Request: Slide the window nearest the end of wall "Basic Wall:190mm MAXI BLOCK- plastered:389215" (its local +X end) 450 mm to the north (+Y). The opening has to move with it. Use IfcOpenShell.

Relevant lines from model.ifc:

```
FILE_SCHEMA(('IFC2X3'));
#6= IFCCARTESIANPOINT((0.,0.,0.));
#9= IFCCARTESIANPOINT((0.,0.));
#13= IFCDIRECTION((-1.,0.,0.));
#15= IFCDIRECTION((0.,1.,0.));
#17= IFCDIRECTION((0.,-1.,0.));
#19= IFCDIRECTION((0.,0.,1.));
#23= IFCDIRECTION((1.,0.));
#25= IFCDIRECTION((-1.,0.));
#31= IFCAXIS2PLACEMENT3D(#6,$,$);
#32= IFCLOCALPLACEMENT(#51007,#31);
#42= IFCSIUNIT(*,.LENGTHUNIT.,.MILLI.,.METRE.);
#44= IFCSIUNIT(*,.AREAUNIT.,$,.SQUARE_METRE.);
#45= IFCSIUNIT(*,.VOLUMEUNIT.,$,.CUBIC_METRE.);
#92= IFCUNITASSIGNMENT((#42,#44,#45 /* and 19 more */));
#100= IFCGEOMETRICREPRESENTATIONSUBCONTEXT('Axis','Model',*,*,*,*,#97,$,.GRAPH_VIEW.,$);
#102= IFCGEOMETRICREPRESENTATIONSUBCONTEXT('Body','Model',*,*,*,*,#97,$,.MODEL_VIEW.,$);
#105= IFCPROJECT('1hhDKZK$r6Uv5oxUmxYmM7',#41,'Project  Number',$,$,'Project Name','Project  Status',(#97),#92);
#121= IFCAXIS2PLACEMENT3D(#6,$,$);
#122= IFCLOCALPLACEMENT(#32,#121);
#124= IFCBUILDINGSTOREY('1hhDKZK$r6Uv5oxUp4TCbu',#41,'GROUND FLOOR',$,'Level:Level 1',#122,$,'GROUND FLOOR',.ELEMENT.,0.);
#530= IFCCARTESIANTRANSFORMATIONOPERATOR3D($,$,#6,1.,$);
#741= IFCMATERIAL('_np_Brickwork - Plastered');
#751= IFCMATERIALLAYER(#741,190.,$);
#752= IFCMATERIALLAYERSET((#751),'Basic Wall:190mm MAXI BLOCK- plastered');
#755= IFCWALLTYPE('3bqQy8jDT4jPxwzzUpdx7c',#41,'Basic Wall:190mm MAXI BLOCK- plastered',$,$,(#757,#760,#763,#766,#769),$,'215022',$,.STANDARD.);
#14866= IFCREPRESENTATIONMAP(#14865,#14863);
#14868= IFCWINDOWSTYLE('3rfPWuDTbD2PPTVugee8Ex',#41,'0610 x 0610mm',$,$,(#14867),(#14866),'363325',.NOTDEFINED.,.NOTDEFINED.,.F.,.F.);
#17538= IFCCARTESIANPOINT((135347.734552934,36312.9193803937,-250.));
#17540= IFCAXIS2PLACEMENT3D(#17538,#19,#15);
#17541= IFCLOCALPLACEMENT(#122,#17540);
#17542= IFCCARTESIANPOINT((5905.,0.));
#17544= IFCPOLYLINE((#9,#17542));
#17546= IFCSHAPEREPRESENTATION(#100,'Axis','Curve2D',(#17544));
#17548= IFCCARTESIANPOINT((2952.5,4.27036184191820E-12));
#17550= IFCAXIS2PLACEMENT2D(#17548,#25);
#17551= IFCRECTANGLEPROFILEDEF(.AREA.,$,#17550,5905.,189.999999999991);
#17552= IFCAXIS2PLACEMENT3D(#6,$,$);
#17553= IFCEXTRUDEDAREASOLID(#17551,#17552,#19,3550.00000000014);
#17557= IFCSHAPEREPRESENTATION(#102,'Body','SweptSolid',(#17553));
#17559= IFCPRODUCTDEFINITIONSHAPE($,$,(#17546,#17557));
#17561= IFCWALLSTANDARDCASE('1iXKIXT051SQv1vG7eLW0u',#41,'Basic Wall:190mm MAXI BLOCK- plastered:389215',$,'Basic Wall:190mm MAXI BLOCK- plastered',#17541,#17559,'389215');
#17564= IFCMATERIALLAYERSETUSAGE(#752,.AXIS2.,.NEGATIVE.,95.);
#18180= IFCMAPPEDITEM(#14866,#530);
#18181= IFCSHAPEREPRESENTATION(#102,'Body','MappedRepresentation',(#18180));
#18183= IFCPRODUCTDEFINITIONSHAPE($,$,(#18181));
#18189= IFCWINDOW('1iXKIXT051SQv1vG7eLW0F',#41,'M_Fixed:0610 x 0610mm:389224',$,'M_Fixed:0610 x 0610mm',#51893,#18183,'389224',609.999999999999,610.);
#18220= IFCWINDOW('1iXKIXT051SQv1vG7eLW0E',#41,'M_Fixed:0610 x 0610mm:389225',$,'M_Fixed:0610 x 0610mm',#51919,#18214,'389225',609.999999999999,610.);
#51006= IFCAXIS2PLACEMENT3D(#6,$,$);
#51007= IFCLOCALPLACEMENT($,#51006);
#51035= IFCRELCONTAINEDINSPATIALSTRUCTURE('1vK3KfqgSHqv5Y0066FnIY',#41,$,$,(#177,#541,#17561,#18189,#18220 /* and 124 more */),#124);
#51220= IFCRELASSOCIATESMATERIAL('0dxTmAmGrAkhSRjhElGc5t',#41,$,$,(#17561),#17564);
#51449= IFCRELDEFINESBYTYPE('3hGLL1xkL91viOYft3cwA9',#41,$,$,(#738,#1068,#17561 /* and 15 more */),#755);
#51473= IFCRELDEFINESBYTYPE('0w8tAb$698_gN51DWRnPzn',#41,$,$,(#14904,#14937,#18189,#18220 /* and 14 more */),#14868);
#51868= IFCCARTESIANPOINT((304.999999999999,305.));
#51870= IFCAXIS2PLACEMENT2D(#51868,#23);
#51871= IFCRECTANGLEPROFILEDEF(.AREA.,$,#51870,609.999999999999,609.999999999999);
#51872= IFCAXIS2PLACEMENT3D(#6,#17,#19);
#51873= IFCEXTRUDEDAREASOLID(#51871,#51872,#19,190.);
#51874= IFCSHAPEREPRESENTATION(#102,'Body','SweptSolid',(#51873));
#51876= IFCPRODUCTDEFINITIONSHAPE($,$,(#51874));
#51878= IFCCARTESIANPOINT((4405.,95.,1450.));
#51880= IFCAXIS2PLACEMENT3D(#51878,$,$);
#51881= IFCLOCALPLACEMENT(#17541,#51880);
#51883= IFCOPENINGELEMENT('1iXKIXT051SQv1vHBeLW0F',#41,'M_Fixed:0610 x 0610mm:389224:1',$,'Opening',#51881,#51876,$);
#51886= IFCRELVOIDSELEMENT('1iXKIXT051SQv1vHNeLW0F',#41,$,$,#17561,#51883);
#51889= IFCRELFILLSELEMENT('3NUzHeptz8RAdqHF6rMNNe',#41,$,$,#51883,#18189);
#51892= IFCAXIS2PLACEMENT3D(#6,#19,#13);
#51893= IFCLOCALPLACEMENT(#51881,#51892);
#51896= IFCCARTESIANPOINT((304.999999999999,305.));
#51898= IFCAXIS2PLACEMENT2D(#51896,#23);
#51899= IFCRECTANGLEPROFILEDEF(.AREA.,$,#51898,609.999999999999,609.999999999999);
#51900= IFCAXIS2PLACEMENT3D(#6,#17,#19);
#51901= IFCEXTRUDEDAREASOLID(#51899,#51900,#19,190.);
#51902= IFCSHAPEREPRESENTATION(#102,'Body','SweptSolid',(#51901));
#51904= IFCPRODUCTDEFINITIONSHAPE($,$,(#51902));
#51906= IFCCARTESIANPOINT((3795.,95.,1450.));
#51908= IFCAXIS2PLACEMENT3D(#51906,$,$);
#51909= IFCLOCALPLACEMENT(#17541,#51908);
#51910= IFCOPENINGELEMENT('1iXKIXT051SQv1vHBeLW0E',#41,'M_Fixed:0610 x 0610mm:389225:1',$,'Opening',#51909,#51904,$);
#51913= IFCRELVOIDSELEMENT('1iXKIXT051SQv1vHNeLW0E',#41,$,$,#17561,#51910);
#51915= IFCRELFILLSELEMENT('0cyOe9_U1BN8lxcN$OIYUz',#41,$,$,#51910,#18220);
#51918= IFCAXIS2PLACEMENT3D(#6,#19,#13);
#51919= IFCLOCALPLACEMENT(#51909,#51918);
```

```python
import ifcopenshell
import ifcopenshell.api.geometry
import ifcopenshell.util.placement

model = ifcopenshell.open("model.ifc")

window = model.by_guid("1iXKIXT051SQv1vG7eLW0F")
opening = window.FillsVoids[0].RelatingOpeningElement
wall = opening.VoidsElements[0].RelatingBuildingElement

wall_matrix = ifcopenshell.util.placement.get_local_placement(wall.ObjectPlacement)
shift = wall_matrix[:3, 0] * 450.0
before = ifcopenshell.util.placement.get_local_placement(window.ObjectPlacement)[:3, 3].copy()

# The window is placed relative to its opening, so it follows when the opening moves.
matrix = ifcopenshell.util.placement.get_local_placement(opening.ObjectPlacement)
matrix[:3, 3] += shift
ifcopenshell.api.geometry.edit_object_placement(
    model, product=opening, matrix=matrix, is_si=False, should_transform_children=True
)

after = ifcopenshell.util.placement.get_local_placement(window.ObjectPlacement)[:3, 3]
print("window moved by", (after - before).round(3) + 0.0)

model.write("model_updated.ifc")
```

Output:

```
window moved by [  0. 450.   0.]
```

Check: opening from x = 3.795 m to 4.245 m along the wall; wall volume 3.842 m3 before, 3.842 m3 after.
